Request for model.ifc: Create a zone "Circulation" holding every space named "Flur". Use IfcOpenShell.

First a look at what the model holds.

```python
import ifcopenshell

model = ifcopenshell.open("model.ifc")
print(model.schema)
seen = {}
for space in model.by_type("IfcSpace"):
    seen[space.LongName] = seen.get(space.LongName, 0) + 1
for name, count in sorted(seen.items(), key=str):
    print(count, "x", name)
print("zones:", [z.Name for z in model.by_type("IfcZone")][:20])
```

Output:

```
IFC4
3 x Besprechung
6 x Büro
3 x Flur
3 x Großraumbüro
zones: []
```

```python
import ifcopenshell
import ifcopenshell.api.group
import ifcopenshell.api.root

model = ifcopenshell.open("model.ifc")

names = {"Flur"}
spaces = [s for s in model.by_type("IfcSpace") if s.LongName in names]

zone = ifcopenshell.api.root.create_entity(model, ifc_class="IfcZone", name="Circulation")
ifcopenshell.api.group.assign_group(model, products=spaces, group=zone)
print(len(spaces), "spaces in", zone.Name)

model.write("model-out.ifc")
```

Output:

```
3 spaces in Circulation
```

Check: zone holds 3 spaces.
